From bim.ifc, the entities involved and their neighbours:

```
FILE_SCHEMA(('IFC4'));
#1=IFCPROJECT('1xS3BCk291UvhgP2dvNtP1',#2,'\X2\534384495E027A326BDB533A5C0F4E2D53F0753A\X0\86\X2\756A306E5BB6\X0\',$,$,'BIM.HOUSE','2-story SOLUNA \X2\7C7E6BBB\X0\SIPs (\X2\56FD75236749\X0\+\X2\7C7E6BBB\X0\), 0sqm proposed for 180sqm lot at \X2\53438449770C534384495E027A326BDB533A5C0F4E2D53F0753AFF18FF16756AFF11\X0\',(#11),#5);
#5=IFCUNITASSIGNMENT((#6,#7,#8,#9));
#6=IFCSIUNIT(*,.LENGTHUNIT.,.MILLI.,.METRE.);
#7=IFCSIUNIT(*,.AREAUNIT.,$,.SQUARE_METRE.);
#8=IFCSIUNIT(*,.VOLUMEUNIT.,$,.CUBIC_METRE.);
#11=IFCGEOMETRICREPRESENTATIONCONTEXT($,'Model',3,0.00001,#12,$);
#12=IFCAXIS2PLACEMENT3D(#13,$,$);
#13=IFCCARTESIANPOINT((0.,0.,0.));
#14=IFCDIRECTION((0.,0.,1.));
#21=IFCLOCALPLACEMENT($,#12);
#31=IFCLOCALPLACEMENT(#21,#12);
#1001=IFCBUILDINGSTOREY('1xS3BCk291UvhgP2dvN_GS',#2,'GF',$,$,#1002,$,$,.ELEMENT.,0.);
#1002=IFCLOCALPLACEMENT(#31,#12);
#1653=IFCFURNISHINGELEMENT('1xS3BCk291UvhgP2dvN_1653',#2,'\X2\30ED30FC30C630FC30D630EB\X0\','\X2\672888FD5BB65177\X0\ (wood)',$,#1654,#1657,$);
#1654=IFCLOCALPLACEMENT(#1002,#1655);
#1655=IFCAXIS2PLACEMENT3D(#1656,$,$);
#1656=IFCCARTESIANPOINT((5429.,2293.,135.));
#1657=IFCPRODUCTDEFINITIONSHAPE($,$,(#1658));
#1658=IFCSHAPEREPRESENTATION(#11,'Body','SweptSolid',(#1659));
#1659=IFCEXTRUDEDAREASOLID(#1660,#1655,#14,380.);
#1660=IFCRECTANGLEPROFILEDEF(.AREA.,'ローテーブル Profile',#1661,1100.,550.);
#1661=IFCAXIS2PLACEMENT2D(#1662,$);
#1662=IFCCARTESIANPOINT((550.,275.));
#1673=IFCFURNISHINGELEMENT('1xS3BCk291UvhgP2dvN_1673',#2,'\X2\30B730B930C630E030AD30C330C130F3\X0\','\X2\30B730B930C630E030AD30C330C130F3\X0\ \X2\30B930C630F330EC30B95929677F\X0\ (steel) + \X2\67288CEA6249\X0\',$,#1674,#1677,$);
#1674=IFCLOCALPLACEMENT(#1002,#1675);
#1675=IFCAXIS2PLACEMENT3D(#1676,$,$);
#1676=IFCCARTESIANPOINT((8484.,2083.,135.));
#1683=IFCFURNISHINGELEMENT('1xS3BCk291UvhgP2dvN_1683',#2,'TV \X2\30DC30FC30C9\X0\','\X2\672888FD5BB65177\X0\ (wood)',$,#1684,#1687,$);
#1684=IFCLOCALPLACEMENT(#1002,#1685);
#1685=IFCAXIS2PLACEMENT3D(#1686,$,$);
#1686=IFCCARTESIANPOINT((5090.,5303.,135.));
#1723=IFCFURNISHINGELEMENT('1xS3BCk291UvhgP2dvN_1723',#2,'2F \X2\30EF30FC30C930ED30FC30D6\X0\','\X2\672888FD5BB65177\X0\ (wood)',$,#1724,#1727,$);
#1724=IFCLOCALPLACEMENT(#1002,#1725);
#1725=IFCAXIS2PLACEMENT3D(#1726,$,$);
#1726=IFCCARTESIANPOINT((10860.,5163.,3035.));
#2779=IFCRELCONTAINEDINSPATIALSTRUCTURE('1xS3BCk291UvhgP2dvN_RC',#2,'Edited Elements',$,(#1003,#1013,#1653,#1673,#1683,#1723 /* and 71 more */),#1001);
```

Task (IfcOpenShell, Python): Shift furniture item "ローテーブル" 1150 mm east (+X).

```python
import ifcopenshell
import ifcopenshell.api.geometry
import ifcopenshell.util.placement
import ifcopenshell.util.unit

model = ifcopenshell.open("bim.ifc")
unit_scale = ifcopenshell.util.unit.calculate_unit_scale(model)

item = model.by_guid("1xS3BCk291UvhgP2dvN_1653")
matrix = ifcopenshell.util.placement.get_local_placement(item.ObjectPlacement)
matrix[0, 3] += 1.15 / unit_scale
ifcopenshell.api.geometry.edit_object_placement(model, product=item, matrix=matrix, is_si=False)

print(ifcopenshell.util.placement.get_local_placement(item.ObjectPlacement).round(3) + 0.0)

model.write("bim_rev.ifc")
```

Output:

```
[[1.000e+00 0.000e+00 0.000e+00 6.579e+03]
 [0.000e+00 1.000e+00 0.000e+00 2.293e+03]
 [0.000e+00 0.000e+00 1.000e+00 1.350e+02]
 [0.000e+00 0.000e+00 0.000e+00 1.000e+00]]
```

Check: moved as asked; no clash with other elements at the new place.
